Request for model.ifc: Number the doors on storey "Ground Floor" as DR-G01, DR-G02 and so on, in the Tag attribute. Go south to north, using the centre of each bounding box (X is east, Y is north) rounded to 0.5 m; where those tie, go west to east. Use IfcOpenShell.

First a look at what the model holds.

```python
import ifcopenshell
import ifcopenshell.util.element
import ifcopenshell.util.placement

model = ifcopenshell.open("model.ifc")
print(model.schema)
storey = next(s for s in model.by_type("IfcBuildingStorey") if s.Name == "Ground Floor")
doors = [e for e in ifcopenshell.util.element.get_decomposition(storey) if e.is_a("IfcDoor")]
for e in sorted(doors, key=lambda e: e.id()):
    origin = ifcopenshell.util.placement.get_local_placement(e.ObjectPlacement)[:3, 3]
    print(e.id(), e.Tag, e.Name, origin.round(2) + 0.0, sep=" | ")
```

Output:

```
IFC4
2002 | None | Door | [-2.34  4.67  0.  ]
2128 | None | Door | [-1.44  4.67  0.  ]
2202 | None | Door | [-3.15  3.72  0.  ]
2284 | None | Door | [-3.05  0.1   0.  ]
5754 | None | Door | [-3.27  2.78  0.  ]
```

```python
import ifcopenshell
import ifcopenshell.geom
import ifcopenshell.util.element
import ifcopenshell.util.shape

model = ifcopenshell.open("model.ifc")
settings = ifcopenshell.geom.settings()
settings.set("use-world-coords", True)


def centre(element):
    shape = ifcopenshell.geom.create_shape(settings, element)
    return ifcopenshell.util.shape.get_bbox_centroid(shape.geometry)


storey = next(s for s in model.by_type("IfcBuildingStorey") if s.Name == "Ground Floor")
doors = [e for e in ifcopenshell.util.element.get_decomposition(storey) if e.is_a("IfcDoor")]

# Insertion points can sit at a corner or the storey origin, so sort by the geometry (in metres).
centres = {e: centre(e) for e in doors}
doors.sort(key=lambda e: (round(centres[e][1] / 0.5), centres[e][0]))

for i, e in enumerate(doors, start=1):
    number = f"DR-G{i:02d}"
    e.Tag = number
    print(e.id(), number)

model.write("model_updated.ifc")
```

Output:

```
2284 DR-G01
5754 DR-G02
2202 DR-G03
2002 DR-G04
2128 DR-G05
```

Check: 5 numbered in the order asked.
